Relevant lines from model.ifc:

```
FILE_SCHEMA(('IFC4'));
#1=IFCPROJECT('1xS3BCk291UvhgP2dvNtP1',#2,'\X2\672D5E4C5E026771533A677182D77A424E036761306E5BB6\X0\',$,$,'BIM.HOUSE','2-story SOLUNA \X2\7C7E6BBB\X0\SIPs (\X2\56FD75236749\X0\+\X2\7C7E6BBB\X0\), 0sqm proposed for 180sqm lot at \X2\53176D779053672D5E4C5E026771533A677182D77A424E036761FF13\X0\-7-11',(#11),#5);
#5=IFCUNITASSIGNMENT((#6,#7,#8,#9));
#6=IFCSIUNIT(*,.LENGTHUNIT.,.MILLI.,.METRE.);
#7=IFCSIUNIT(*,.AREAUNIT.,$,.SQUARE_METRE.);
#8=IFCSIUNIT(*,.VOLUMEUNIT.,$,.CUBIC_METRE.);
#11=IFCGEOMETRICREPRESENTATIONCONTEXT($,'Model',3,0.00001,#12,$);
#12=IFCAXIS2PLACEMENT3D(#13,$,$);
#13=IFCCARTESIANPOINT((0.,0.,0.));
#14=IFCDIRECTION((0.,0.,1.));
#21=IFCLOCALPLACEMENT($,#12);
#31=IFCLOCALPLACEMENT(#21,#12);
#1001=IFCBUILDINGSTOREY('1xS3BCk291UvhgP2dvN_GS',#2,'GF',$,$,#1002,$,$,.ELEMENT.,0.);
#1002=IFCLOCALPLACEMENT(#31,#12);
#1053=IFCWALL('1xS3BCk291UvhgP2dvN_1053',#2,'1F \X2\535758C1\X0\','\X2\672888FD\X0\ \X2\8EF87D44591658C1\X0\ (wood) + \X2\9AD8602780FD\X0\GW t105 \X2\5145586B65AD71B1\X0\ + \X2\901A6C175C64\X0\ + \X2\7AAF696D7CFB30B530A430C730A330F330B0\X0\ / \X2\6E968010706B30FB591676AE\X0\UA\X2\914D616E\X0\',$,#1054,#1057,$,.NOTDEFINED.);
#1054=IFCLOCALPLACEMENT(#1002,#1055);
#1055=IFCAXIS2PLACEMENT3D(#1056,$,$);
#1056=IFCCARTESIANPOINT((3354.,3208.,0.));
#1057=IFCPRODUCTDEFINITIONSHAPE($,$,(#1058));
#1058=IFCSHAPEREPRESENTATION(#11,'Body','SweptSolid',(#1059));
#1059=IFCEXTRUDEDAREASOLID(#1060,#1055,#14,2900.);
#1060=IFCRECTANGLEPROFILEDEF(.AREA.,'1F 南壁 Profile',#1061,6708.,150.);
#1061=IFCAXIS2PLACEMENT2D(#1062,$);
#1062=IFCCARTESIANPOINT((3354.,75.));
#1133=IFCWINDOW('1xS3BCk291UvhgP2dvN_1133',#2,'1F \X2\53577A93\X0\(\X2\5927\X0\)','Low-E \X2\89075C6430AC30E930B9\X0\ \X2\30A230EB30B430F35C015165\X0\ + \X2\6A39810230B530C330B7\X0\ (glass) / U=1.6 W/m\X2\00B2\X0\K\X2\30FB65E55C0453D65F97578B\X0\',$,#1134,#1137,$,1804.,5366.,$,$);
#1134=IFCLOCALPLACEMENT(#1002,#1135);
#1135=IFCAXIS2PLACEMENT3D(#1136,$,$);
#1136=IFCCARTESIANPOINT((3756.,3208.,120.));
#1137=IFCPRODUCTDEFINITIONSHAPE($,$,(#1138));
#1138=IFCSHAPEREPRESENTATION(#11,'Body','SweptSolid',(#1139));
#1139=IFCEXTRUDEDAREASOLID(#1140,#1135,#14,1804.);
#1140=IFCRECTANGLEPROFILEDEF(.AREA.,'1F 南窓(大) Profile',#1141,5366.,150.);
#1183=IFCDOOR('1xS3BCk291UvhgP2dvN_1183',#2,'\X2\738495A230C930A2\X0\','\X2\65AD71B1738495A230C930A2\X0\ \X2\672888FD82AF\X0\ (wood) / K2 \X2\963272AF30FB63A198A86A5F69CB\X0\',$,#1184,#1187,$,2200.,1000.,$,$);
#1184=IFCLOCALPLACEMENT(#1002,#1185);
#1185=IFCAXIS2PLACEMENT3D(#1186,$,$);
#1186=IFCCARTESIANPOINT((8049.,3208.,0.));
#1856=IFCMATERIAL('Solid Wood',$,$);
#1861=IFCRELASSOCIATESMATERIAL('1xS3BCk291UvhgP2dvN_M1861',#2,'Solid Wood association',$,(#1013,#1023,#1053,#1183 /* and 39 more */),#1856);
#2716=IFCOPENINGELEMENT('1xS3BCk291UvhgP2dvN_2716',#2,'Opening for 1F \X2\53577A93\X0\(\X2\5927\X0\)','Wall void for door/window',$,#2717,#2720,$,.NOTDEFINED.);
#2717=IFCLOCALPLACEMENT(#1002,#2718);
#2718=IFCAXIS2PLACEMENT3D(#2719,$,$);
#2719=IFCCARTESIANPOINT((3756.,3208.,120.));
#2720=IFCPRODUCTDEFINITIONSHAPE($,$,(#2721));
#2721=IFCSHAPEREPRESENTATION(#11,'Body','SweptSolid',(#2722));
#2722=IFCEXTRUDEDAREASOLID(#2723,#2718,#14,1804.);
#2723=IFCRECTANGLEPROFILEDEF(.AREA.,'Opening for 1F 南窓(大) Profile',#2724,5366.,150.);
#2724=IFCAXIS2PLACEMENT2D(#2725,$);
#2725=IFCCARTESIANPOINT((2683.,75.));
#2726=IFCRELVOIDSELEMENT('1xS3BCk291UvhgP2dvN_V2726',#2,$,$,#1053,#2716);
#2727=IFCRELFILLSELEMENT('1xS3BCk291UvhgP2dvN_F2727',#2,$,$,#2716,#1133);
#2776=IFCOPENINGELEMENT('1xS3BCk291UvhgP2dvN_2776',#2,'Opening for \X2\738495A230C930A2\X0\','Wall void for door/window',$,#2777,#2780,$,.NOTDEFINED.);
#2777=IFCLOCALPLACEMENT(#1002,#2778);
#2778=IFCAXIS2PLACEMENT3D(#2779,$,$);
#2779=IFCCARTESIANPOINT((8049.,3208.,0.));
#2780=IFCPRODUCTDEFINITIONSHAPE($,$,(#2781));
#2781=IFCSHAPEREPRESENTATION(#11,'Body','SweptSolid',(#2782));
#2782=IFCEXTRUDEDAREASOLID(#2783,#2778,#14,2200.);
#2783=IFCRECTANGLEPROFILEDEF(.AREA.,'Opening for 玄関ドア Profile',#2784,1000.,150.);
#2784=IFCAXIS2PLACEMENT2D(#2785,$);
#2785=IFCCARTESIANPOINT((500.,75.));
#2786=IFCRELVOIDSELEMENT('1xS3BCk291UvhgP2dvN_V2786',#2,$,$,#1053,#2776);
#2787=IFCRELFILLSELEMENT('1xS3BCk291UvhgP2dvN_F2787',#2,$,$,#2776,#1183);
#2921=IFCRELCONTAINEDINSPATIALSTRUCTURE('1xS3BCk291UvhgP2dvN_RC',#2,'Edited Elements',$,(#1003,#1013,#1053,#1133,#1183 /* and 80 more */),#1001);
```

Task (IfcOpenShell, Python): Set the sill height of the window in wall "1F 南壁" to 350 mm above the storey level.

```python
import numpy as np
import ifcopenshell
import ifcopenshell.api.geometry
import ifcopenshell.geom
import ifcopenshell.util.element
import ifcopenshell.util.placement
import ifcopenshell.util.shape
import ifcopenshell.util.unit

model = ifcopenshell.open("model.ifc")
unit_scale = ifcopenshell.util.unit.calculate_unit_scale(model)

window = model.by_guid("1xS3BCk291UvhgP2dvN_1133")
opening = window.FillsVoids[0].RelatingOpeningElement
storey = ifcopenshell.util.element.get_container(window, ifc_class="IfcBuildingStorey")
level = ifcopenshell.util.placement.get_local_placement(storey.ObjectPlacement)[2, 3]

# The opening's origin need not be at the sill, so measure its lowest point.
shape = ifcopenshell.geom.create_shape(ifcopenshell.geom.settings(), opening)
bottom = ifcopenshell.util.shape.get_shape_bottom_elevation(shape, shape.geometry) / unit_scale
dz = level + 350.0 - bottom

shift = np.array([0.0, 0.0, dz])
# The window is not placed relative to its opening, so move both.
for product in (opening, window):
    matrix = ifcopenshell.util.placement.get_local_placement(product.ObjectPlacement)
    matrix[:3, 3] += shift
    ifcopenshell.api.geometry.edit_object_placement(model, product=product, matrix=matrix, is_si=False)

print(f"moved by {dz * unit_scale:+.3f} m")

model.write("model_updated.ifc")
```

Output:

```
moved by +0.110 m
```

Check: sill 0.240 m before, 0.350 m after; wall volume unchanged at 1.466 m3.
